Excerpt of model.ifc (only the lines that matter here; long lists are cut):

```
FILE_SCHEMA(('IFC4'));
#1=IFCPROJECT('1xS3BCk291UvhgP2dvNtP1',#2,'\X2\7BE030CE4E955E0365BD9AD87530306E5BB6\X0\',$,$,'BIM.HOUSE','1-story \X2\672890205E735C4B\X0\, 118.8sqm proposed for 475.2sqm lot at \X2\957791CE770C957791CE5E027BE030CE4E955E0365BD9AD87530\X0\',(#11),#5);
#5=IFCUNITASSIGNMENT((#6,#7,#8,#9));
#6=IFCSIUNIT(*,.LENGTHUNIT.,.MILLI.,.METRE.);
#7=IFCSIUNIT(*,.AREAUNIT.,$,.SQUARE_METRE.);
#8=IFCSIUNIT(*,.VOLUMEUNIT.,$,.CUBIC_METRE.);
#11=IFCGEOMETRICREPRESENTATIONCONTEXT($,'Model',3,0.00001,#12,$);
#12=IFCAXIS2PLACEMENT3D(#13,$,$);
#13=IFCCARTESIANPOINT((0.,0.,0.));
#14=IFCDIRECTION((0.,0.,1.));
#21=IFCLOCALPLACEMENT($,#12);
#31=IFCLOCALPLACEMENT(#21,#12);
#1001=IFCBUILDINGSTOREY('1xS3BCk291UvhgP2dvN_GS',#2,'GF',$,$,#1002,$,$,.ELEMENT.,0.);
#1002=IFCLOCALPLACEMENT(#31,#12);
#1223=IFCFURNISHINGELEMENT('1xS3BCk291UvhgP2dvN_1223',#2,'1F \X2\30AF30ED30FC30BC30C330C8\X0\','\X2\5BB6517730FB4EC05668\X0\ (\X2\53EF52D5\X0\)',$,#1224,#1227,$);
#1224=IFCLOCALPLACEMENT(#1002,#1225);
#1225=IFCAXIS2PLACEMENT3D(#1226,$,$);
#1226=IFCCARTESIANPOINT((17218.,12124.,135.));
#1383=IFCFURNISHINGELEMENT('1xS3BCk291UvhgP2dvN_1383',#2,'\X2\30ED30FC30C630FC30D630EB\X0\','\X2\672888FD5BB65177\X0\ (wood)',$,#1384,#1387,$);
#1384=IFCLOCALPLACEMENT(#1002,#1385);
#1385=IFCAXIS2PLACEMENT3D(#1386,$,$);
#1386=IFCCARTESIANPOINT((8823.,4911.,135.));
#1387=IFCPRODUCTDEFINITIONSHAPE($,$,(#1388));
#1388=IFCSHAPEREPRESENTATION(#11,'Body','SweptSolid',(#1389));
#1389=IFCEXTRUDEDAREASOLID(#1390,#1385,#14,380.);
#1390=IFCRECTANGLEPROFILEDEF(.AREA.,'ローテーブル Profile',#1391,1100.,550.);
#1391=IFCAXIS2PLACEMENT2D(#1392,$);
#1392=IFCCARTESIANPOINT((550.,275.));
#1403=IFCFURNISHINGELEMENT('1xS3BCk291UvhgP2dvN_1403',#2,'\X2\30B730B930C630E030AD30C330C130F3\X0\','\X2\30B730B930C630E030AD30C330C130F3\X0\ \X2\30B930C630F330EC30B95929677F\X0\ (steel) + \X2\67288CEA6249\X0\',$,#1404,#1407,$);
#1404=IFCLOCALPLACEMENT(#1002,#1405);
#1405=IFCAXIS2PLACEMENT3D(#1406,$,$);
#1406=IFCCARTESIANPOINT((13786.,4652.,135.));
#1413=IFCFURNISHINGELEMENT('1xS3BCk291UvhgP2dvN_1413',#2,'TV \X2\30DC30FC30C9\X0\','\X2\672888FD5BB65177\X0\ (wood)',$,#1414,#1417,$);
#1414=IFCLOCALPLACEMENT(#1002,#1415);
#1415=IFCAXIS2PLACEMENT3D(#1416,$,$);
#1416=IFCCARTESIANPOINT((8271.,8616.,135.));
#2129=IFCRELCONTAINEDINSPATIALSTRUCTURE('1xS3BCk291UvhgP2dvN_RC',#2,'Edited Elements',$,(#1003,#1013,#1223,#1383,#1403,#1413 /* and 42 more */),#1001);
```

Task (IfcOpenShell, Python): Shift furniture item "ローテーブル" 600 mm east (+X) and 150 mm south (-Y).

```python
import ifcopenshell
import ifcopenshell.api.geometry
import ifcopenshell.util.placement
import ifcopenshell.util.unit

model = ifcopenshell.open("model.ifc")
unit_scale = ifcopenshell.util.unit.calculate_unit_scale(model)

item = model.by_guid("1xS3BCk291UvhgP2dvN_1383")
matrix = ifcopenshell.util.placement.get_local_placement(item.ObjectPlacement)
matrix[0, 3] += 0.6 / unit_scale
matrix[1, 3] -= 0.15 / unit_scale
ifcopenshell.api.geometry.edit_object_placement(model, product=item, matrix=matrix, is_si=False)

print(ifcopenshell.util.placement.get_local_placement(item.ObjectPlacement).round(3) + 0.0)

model.write("model_edited.ifc")
```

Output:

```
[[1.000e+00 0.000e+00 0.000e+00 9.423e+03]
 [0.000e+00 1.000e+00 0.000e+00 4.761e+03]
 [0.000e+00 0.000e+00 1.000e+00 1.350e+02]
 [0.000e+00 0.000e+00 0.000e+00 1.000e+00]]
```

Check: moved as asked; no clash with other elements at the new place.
